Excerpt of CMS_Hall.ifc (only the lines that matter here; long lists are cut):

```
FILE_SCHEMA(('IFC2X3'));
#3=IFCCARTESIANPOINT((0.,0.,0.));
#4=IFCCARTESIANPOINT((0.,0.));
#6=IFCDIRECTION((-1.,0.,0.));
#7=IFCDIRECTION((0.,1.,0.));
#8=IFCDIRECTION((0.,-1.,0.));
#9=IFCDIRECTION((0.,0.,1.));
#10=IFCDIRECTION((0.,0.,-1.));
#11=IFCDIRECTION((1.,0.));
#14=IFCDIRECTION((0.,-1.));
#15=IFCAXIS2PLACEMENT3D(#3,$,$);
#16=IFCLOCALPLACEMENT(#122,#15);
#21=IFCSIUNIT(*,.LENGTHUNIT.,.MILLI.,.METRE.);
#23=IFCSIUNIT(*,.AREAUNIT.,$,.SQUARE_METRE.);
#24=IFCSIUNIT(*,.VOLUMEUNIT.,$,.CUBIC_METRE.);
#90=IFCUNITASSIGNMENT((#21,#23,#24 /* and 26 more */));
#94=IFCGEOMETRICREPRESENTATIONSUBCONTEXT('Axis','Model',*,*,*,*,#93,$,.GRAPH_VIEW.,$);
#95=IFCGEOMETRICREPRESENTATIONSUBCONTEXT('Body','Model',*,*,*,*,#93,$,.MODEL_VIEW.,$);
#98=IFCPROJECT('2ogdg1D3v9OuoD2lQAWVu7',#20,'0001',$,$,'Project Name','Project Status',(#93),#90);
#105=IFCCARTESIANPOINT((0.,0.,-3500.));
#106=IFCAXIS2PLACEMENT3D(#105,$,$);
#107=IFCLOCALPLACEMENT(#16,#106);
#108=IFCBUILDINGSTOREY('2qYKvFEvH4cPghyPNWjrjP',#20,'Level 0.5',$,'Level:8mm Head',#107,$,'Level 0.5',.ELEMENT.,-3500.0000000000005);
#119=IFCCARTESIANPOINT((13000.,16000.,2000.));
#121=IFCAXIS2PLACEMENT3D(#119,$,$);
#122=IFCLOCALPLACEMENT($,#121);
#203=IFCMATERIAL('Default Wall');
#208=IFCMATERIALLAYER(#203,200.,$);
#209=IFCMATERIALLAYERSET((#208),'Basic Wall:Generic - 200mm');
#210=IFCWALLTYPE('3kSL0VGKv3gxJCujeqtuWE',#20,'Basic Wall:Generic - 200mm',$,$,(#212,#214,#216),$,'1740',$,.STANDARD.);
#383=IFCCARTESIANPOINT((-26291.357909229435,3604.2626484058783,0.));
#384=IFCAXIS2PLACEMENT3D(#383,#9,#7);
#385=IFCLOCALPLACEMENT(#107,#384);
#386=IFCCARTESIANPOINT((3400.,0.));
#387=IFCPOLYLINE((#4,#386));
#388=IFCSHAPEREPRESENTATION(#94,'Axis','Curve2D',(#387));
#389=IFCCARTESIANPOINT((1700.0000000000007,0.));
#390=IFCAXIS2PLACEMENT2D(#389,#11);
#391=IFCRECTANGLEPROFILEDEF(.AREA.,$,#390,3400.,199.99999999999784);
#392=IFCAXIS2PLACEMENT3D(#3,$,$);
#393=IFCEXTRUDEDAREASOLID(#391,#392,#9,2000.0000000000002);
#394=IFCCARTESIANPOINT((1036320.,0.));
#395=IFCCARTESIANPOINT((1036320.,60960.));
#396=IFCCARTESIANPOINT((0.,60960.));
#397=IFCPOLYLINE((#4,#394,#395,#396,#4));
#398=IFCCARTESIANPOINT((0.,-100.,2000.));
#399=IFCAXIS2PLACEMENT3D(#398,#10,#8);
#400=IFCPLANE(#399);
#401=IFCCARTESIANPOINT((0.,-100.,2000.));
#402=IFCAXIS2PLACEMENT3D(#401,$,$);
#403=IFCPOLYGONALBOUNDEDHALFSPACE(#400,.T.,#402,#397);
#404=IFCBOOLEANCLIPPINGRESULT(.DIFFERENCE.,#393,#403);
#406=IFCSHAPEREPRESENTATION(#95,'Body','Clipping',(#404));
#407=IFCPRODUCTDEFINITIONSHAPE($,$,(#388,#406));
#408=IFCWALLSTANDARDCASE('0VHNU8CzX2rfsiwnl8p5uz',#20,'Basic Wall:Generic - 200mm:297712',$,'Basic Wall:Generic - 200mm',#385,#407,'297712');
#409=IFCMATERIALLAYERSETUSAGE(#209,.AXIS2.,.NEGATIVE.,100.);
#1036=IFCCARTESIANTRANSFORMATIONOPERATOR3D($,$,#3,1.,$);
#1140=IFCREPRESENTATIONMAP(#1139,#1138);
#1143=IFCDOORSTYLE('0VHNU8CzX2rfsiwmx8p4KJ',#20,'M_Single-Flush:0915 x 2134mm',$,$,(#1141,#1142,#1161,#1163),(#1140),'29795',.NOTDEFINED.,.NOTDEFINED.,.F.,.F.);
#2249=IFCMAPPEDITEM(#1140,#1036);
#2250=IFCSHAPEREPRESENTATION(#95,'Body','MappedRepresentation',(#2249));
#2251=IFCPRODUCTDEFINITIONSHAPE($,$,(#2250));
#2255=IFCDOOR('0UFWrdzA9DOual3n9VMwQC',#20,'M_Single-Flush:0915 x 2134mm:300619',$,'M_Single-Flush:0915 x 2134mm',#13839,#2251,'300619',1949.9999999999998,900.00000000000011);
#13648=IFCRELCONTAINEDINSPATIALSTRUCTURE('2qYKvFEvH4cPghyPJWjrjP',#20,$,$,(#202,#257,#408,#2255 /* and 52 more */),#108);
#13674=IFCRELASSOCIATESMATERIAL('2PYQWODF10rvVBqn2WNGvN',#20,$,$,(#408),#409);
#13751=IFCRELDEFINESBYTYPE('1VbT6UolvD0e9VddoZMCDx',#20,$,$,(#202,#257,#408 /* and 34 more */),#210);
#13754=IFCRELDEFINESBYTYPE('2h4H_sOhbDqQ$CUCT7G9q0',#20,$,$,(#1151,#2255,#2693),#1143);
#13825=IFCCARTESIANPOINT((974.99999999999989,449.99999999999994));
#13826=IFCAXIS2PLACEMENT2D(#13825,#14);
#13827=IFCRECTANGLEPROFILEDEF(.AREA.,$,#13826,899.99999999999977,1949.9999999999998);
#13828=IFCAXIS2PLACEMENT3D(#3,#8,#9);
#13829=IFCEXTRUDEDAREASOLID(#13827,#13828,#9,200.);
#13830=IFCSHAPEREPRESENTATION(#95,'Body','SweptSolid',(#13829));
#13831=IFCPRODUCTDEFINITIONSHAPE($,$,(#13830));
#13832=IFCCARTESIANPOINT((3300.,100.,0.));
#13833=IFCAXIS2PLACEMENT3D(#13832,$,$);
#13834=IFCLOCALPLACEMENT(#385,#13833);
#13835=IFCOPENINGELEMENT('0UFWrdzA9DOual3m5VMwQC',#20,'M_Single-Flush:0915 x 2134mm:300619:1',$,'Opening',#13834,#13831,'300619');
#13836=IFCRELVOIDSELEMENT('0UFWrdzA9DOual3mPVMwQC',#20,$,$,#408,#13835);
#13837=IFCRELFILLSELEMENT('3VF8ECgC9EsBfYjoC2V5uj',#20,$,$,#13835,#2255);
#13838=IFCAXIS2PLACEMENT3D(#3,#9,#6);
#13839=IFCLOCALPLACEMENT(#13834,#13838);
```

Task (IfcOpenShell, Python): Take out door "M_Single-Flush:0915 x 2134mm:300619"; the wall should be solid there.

```python
import ifcopenshell
import ifcopenshell.api.feature
import ifcopenshell.api.root
import ifcopenshell.geom
import ifcopenshell.util.shape

model = ifcopenshell.open("CMS_Hall.ifc")
settings = ifcopenshell.geom.settings()


def volume(element):
    """Net volume in cubic metres, openings subtracted."""
    shape = ifcopenshell.geom.create_shape(settings, element)
    return ifcopenshell.util.shape.get_volume(shape.geometry)


door = model.by_guid("0UFWrdzA9DOual3n9VMwQC")
opening = door.FillsVoids[0].RelatingOpeningElement
wall = opening.VoidsElements[0].RelatingBuildingElement
before = volume(wall)

ifcopenshell.api.root.remove_product(model, product=door)
ifcopenshell.api.feature.remove_feature(model, feature=opening)

after = volume(wall)

print(f"wall volume {before:.3f} -> {after:.3f} m3")

model.write("CMS_Hall_v2.ifc")
```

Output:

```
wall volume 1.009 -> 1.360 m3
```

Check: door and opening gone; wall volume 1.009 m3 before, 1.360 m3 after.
